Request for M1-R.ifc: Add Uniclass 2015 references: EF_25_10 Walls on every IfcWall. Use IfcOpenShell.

First a look at what the model holds.

```python
import ifcopenshell

model = ifcopenshell.open("M1-R.ifc")
print(model.schema)
print("classifications:", [c.Name for c in model.by_type("IfcClassification")])
for ifc_class in ("IfcDoor", "IfcRoof", "IfcStair", "IfcWall", "IfcWindow"):
    print(ifc_class, len(model.by_type(ifc_class)))
```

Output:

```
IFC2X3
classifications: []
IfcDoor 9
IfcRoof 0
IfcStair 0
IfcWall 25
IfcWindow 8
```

```python
import ifcopenshell
import ifcopenshell.api.classification

model = ifcopenshell.open("M1-R.ifc")

# IFC2X3 requires Source and Edition and has no link from the project to the system.
system = model.create_entity("IfcClassification", Source="NBS", Edition="2015", Name="Uniclass 2015")

codes = {
    "IfcWall": ("EF_25_10", "Walls"),
}
for ifc_class, (code, name) in codes.items():
    products = model.by_type(ifc_class)
    ifcopenshell.api.classification.add_reference(
        model, products=products, classification=system, identification=code, name=name
    )
    print(code, len(products))

model.write("M1-R_edited.ifc")
```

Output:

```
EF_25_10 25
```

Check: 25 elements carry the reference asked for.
